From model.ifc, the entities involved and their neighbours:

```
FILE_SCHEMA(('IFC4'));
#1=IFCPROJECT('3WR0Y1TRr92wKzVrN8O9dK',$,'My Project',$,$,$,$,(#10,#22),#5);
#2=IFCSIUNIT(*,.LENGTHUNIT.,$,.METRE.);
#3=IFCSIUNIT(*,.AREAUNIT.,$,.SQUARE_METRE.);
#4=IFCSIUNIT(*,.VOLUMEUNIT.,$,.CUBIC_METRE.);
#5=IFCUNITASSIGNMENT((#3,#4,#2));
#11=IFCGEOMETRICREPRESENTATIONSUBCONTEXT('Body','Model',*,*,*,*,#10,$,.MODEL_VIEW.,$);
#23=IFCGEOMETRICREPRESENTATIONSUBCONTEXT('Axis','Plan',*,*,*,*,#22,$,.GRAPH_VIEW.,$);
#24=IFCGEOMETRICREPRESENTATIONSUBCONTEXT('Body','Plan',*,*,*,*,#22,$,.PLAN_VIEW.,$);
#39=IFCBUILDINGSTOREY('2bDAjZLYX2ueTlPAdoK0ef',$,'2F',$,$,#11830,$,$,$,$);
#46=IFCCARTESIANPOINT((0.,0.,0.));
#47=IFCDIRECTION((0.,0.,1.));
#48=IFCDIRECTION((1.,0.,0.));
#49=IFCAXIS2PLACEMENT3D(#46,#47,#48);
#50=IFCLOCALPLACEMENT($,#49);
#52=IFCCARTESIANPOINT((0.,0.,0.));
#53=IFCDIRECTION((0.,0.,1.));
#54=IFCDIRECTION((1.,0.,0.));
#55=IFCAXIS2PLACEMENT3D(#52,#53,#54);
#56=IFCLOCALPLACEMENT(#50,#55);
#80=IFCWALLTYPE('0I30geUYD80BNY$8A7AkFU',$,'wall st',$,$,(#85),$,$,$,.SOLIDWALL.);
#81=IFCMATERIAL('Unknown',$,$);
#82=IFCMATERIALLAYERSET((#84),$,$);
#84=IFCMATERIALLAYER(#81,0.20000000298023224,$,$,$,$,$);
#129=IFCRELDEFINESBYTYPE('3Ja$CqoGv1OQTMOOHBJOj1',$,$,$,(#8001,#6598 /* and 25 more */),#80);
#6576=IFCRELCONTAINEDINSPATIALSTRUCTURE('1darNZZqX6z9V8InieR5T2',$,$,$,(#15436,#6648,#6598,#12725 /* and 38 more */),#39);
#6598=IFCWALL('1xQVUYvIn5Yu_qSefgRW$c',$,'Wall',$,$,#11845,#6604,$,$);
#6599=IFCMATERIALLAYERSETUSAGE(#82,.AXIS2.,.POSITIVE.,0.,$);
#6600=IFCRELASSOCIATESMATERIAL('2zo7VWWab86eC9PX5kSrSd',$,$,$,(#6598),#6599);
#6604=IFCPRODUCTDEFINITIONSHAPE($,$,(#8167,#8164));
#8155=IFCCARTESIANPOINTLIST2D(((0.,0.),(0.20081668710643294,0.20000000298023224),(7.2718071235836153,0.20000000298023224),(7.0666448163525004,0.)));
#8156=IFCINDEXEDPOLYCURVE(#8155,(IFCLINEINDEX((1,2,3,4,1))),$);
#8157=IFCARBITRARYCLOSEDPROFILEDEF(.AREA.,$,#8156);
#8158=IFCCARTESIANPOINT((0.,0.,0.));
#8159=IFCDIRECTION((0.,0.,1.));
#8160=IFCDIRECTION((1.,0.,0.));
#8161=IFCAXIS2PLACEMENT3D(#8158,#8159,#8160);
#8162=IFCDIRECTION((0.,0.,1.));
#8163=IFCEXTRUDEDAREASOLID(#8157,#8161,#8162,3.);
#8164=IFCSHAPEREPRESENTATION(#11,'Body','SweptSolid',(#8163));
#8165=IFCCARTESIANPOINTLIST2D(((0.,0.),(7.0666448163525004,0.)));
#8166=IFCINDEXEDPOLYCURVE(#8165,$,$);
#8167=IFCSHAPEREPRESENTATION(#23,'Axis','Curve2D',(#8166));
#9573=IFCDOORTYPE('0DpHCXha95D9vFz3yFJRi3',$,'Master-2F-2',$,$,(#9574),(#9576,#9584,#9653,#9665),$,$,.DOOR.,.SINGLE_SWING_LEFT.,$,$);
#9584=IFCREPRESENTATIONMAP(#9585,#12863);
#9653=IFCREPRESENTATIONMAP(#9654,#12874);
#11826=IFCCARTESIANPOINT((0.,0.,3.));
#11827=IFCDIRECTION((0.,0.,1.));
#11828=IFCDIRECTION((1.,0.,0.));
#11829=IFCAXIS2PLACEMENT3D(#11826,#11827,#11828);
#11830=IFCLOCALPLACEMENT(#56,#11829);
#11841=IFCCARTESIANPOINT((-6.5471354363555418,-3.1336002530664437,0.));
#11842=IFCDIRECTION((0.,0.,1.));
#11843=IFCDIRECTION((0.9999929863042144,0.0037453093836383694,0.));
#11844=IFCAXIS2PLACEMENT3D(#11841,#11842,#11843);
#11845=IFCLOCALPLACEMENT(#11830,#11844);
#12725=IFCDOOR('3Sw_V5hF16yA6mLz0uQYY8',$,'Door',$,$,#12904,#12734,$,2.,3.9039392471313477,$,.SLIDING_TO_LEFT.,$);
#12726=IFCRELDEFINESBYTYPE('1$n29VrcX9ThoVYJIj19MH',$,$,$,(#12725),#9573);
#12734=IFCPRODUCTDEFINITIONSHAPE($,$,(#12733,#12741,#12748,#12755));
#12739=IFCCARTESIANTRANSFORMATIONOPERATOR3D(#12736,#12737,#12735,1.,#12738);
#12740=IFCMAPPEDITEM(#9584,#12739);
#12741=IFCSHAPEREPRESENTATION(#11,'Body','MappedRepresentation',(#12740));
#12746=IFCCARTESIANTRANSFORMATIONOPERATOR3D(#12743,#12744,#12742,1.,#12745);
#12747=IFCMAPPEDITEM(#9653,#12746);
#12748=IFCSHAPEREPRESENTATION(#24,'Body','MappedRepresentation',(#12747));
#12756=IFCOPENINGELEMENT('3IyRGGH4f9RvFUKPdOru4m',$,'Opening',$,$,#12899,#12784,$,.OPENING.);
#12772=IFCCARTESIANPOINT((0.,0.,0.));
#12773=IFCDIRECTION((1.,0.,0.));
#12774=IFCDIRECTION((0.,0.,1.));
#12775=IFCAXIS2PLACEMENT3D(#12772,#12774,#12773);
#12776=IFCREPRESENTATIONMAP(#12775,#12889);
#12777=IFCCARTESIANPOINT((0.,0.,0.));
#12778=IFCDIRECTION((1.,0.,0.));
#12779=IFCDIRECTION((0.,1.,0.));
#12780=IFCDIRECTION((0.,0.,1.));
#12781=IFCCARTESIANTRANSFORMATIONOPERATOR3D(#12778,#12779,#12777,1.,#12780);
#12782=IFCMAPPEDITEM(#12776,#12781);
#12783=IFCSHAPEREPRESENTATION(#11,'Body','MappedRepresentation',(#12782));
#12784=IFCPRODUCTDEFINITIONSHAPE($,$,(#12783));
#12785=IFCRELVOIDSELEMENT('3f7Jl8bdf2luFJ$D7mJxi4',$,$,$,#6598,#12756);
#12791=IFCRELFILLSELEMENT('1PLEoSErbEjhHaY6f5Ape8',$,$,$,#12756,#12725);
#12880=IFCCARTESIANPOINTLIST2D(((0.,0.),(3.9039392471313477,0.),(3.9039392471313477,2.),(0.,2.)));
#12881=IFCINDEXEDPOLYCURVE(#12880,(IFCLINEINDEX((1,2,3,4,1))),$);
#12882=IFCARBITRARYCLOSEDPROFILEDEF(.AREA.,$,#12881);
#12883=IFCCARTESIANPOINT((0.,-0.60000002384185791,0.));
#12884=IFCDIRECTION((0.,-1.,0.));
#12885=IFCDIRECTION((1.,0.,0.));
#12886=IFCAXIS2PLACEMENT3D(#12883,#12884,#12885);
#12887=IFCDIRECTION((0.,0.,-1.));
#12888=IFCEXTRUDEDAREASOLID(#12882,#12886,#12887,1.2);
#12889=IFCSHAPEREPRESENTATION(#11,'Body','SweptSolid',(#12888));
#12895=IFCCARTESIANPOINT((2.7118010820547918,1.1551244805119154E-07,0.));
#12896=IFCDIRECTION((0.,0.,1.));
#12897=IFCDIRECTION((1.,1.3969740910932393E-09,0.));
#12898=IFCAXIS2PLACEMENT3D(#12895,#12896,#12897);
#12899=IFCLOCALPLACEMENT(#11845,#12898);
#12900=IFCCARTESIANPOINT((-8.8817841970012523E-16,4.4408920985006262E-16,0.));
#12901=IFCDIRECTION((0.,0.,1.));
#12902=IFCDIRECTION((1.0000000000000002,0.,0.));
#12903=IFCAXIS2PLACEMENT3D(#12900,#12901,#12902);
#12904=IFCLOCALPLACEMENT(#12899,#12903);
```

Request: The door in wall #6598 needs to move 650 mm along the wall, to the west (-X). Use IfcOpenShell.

```python
import ifcopenshell
import ifcopenshell.api.geometry
import ifcopenshell.util.placement

model = ifcopenshell.open("model.ifc")

door = model.by_guid("3Sw_V5hF16yA6mLz0uQYY8")
opening = door.FillsVoids[0].RelatingOpeningElement
wall = opening.VoidsElements[0].RelatingBuildingElement

wall_matrix = ifcopenshell.util.placement.get_local_placement(wall.ObjectPlacement)
shift = wall_matrix[:3, 0] * -0.65
before = ifcopenshell.util.placement.get_local_placement(door.ObjectPlacement)[:3, 3].copy()

# The door is placed relative to its opening, so it follows when the opening moves.
matrix = ifcopenshell.util.placement.get_local_placement(opening.ObjectPlacement)
matrix[:3, 3] += shift
ifcopenshell.api.geometry.edit_object_placement(
    model, product=opening, matrix=matrix, is_si=False, should_transform_children=True
)

after = ifcopenshell.util.placement.get_local_placement(door.ObjectPlacement)[:3, 3]
print("door moved by", (after - before).round(3) + 0.0)

model.write("model-out.ifc")
```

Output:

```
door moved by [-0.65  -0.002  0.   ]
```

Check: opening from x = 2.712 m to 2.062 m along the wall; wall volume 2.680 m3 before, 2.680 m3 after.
